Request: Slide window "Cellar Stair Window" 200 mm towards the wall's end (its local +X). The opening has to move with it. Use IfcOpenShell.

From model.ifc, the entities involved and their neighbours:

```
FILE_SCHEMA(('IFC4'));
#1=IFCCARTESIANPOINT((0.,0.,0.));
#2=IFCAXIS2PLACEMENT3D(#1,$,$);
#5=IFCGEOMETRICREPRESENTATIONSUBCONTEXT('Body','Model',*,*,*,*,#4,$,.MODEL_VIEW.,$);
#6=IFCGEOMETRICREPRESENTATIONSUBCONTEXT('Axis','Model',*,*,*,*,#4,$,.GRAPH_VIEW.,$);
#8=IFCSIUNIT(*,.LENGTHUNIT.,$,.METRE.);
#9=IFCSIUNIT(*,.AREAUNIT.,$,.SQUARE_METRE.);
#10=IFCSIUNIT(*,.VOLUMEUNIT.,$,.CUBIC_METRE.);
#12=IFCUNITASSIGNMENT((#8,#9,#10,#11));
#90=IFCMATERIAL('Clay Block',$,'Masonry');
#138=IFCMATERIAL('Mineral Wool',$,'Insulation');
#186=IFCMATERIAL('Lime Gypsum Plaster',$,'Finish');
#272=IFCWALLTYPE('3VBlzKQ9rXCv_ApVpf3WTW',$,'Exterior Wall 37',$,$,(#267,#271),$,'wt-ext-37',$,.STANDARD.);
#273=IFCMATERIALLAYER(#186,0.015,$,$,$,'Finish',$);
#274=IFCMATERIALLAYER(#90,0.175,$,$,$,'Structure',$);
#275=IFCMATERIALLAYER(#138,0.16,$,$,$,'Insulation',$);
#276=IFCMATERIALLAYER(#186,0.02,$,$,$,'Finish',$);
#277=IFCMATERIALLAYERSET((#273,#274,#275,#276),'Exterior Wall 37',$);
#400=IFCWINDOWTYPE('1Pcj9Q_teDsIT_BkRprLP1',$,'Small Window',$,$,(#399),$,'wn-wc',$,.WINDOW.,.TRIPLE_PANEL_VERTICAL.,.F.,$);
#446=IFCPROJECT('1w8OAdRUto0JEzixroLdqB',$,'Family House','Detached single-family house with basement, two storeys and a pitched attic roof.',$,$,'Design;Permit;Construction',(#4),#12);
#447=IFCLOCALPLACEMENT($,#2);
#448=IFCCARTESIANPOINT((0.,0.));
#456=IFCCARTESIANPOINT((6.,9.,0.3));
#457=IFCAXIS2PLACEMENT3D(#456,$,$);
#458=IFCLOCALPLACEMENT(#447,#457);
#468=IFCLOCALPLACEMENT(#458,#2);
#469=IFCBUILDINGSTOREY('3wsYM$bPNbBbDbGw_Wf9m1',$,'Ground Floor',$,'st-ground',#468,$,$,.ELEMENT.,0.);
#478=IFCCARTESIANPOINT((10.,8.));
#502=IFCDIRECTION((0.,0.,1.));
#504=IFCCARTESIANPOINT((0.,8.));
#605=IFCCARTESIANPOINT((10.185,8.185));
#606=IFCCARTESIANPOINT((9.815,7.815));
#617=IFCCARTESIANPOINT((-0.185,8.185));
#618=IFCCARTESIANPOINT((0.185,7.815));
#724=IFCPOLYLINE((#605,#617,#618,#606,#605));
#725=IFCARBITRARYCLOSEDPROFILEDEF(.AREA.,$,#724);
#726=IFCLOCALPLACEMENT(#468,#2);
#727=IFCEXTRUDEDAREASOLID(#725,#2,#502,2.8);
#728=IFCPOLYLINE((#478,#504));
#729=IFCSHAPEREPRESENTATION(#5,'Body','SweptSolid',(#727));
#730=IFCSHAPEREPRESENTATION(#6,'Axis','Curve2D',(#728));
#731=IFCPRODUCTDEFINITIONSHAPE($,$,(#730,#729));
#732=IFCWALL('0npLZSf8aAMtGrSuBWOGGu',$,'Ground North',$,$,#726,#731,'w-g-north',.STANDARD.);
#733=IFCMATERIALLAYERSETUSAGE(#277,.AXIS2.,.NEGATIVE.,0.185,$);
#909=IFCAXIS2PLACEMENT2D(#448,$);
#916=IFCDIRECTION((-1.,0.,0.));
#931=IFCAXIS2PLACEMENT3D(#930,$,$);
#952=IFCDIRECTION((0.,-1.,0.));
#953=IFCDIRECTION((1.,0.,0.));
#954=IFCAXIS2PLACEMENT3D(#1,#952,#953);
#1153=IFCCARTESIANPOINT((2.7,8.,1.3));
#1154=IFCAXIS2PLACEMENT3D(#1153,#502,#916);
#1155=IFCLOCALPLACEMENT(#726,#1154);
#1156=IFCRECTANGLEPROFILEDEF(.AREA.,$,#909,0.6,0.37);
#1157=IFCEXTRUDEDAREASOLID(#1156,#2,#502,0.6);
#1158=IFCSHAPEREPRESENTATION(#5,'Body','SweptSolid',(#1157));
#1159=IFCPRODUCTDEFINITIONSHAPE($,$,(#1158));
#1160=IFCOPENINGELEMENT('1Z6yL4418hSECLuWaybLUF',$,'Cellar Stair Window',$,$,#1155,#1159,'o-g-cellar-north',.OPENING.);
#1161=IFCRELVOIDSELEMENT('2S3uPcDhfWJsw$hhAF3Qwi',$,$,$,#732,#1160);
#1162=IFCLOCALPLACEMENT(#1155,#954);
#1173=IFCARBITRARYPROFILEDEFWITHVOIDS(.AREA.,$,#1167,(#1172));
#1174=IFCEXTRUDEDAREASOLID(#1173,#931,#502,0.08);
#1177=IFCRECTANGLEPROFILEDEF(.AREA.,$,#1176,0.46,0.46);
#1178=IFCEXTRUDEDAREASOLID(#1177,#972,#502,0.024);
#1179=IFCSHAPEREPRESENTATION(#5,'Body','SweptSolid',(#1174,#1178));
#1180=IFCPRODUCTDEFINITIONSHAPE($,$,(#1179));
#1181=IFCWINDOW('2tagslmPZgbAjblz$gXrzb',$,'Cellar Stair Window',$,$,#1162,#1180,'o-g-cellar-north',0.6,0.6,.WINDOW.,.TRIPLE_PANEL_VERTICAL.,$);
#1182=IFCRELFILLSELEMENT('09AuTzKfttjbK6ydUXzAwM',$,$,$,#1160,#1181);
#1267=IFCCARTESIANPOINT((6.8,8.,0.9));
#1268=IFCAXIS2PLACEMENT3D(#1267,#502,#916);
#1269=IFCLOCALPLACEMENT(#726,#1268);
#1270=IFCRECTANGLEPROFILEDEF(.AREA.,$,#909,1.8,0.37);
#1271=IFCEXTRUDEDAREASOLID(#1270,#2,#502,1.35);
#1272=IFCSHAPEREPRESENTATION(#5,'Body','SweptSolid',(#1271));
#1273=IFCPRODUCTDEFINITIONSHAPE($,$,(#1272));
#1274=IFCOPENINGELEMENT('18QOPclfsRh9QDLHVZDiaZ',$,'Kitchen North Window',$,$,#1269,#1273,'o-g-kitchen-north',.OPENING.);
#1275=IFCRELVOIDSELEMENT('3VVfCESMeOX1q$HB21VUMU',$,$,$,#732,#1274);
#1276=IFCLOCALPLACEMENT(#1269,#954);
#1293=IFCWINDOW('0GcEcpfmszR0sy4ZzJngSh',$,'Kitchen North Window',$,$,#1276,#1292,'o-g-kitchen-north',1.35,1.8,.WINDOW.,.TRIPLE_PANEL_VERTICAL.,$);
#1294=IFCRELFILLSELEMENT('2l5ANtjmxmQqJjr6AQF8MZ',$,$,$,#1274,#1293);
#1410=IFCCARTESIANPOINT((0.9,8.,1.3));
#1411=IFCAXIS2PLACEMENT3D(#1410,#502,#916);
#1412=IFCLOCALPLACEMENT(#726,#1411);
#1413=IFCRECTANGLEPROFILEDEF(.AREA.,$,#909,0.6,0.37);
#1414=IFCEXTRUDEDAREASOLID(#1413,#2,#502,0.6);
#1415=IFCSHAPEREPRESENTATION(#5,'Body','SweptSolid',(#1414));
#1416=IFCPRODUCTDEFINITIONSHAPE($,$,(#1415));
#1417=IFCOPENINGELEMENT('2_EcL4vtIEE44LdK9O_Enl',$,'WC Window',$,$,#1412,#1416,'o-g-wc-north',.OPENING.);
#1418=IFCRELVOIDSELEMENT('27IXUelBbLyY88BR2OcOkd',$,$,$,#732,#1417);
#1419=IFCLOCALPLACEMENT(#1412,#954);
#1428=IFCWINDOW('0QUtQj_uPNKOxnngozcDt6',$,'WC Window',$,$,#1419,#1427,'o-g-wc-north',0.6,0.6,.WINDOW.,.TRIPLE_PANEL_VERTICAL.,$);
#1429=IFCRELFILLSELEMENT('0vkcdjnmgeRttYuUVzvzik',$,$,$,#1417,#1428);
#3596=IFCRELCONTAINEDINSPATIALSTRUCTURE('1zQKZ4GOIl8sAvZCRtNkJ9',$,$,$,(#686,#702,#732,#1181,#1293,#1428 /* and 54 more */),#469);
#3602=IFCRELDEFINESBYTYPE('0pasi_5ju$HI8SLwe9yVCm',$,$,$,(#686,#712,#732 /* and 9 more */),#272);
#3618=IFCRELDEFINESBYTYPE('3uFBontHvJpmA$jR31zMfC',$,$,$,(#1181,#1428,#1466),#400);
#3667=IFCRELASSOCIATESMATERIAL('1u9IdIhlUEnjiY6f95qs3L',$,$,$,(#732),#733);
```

```python
import ifcopenshell
import ifcopenshell.api.geometry
import ifcopenshell.util.placement

model = ifcopenshell.open("model.ifc")

window = model.by_guid("2tagslmPZgbAjblz$gXrzb")
opening = window.FillsVoids[0].RelatingOpeningElement
wall = opening.VoidsElements[0].RelatingBuildingElement

wall_matrix = ifcopenshell.util.placement.get_local_placement(wall.ObjectPlacement)
shift = wall_matrix[:3, 0] * 0.2
before = ifcopenshell.util.placement.get_local_placement(window.ObjectPlacement)[:3, 3].copy()

# The window is placed relative to its opening, so it follows when the opening moves.
matrix = ifcopenshell.util.placement.get_local_placement(opening.ObjectPlacement)
matrix[:3, 3] += shift
ifcopenshell.api.geometry.edit_object_placement(
    model, product=opening, matrix=matrix, is_si=False, should_transform_children=True
)

after = ifcopenshell.util.placement.get_local_placement(window.ObjectPlacement)[:3, 3]
print("window moved by", (after - before).round(3) + 0.0)

model.write("model-out.ifc")
```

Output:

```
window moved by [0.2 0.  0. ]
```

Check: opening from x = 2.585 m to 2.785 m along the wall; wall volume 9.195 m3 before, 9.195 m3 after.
